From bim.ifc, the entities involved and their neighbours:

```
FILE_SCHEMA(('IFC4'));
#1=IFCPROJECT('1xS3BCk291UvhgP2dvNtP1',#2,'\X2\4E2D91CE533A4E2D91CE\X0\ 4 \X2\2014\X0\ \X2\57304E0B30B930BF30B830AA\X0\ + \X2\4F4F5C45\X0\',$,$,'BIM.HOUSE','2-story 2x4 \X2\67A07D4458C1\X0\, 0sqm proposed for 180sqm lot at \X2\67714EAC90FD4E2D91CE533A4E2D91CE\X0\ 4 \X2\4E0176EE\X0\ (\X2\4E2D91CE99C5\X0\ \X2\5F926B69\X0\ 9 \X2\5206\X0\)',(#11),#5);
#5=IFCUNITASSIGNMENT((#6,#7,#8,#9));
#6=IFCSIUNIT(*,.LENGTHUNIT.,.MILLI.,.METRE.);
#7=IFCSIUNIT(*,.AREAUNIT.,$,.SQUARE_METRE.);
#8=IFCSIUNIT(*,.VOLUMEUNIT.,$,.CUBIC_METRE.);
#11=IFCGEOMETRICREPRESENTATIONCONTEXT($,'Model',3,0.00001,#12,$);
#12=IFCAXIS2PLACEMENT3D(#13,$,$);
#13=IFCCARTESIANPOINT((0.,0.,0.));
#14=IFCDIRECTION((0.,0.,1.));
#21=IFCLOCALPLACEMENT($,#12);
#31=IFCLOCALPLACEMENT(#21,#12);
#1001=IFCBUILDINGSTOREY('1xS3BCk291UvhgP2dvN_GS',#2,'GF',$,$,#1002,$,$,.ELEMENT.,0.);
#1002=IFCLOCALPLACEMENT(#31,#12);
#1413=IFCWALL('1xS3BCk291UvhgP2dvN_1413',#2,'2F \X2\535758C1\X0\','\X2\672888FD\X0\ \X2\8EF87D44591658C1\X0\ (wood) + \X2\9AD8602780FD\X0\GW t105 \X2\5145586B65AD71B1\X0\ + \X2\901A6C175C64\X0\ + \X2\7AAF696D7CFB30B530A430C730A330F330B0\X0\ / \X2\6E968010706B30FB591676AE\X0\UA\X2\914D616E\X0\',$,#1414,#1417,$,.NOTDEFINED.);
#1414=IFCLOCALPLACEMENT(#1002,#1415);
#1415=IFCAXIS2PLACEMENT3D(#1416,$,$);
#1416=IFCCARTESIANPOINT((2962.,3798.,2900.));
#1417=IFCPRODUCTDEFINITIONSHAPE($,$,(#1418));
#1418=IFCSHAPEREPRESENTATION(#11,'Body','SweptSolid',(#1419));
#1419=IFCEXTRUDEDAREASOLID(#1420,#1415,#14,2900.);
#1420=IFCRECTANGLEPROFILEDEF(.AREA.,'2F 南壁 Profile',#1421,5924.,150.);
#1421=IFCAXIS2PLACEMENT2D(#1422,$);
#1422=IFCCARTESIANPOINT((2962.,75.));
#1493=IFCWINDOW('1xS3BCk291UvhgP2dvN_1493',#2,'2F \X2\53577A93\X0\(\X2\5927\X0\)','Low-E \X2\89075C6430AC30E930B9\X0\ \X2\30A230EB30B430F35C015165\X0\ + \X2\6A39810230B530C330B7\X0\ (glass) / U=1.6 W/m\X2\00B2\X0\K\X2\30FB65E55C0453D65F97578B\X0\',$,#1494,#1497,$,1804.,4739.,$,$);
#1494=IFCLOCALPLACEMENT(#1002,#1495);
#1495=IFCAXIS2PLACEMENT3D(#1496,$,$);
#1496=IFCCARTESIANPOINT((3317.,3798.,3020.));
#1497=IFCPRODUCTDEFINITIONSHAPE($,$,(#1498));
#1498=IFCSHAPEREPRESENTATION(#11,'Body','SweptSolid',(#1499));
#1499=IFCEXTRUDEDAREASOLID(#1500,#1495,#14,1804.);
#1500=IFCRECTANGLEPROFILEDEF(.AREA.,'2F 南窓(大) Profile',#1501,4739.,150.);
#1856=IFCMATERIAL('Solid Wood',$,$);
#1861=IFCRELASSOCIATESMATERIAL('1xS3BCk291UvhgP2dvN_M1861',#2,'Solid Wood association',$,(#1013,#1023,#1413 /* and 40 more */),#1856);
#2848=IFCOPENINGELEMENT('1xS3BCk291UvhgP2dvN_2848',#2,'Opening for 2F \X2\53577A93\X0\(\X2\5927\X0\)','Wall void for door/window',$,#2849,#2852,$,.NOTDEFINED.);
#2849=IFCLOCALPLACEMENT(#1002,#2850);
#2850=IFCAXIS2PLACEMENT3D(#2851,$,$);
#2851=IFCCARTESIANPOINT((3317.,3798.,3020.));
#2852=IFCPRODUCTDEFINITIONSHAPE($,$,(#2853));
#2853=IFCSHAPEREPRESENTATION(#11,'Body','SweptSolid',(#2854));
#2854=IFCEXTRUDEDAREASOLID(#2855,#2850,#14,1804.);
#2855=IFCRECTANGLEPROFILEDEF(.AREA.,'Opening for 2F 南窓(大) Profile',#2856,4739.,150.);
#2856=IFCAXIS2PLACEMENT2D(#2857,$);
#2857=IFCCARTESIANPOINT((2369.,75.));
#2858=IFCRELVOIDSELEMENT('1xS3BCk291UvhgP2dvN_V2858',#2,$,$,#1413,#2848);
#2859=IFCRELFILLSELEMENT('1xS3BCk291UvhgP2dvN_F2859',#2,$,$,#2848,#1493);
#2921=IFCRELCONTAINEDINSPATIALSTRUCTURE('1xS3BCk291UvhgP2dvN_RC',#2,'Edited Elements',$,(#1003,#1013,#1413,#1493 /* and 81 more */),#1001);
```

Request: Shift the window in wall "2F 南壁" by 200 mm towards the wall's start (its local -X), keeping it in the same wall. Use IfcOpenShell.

```python
import ifcopenshell
import ifcopenshell.api.geometry
import ifcopenshell.util.placement

model = ifcopenshell.open("bim.ifc")

window = model.by_id(1493)
opening = window.FillsVoids[0].RelatingOpeningElement
wall = opening.VoidsElements[0].RelatingBuildingElement

wall_matrix = ifcopenshell.util.placement.get_local_placement(wall.ObjectPlacement)
shift = wall_matrix[:3, 0] * -200.0
before = ifcopenshell.util.placement.get_local_placement(window.ObjectPlacement)[:3, 3].copy()

# The window is not placed relative to its opening, so move both.
for product in (opening, window):
    matrix = ifcopenshell.util.placement.get_local_placement(product.ObjectPlacement)
    matrix[:3, 3] += shift
    ifcopenshell.api.geometry.edit_object_placement(model, product=product, matrix=matrix, is_si=False)

after = ifcopenshell.util.placement.get_local_placement(window.ObjectPlacement)[:3, 3]
print("window moved by", (after - before).round(3) + 0.0)

model.write("bim_edited.ifc")
```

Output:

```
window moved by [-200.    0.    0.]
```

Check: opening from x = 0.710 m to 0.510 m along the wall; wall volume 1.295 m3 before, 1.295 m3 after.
